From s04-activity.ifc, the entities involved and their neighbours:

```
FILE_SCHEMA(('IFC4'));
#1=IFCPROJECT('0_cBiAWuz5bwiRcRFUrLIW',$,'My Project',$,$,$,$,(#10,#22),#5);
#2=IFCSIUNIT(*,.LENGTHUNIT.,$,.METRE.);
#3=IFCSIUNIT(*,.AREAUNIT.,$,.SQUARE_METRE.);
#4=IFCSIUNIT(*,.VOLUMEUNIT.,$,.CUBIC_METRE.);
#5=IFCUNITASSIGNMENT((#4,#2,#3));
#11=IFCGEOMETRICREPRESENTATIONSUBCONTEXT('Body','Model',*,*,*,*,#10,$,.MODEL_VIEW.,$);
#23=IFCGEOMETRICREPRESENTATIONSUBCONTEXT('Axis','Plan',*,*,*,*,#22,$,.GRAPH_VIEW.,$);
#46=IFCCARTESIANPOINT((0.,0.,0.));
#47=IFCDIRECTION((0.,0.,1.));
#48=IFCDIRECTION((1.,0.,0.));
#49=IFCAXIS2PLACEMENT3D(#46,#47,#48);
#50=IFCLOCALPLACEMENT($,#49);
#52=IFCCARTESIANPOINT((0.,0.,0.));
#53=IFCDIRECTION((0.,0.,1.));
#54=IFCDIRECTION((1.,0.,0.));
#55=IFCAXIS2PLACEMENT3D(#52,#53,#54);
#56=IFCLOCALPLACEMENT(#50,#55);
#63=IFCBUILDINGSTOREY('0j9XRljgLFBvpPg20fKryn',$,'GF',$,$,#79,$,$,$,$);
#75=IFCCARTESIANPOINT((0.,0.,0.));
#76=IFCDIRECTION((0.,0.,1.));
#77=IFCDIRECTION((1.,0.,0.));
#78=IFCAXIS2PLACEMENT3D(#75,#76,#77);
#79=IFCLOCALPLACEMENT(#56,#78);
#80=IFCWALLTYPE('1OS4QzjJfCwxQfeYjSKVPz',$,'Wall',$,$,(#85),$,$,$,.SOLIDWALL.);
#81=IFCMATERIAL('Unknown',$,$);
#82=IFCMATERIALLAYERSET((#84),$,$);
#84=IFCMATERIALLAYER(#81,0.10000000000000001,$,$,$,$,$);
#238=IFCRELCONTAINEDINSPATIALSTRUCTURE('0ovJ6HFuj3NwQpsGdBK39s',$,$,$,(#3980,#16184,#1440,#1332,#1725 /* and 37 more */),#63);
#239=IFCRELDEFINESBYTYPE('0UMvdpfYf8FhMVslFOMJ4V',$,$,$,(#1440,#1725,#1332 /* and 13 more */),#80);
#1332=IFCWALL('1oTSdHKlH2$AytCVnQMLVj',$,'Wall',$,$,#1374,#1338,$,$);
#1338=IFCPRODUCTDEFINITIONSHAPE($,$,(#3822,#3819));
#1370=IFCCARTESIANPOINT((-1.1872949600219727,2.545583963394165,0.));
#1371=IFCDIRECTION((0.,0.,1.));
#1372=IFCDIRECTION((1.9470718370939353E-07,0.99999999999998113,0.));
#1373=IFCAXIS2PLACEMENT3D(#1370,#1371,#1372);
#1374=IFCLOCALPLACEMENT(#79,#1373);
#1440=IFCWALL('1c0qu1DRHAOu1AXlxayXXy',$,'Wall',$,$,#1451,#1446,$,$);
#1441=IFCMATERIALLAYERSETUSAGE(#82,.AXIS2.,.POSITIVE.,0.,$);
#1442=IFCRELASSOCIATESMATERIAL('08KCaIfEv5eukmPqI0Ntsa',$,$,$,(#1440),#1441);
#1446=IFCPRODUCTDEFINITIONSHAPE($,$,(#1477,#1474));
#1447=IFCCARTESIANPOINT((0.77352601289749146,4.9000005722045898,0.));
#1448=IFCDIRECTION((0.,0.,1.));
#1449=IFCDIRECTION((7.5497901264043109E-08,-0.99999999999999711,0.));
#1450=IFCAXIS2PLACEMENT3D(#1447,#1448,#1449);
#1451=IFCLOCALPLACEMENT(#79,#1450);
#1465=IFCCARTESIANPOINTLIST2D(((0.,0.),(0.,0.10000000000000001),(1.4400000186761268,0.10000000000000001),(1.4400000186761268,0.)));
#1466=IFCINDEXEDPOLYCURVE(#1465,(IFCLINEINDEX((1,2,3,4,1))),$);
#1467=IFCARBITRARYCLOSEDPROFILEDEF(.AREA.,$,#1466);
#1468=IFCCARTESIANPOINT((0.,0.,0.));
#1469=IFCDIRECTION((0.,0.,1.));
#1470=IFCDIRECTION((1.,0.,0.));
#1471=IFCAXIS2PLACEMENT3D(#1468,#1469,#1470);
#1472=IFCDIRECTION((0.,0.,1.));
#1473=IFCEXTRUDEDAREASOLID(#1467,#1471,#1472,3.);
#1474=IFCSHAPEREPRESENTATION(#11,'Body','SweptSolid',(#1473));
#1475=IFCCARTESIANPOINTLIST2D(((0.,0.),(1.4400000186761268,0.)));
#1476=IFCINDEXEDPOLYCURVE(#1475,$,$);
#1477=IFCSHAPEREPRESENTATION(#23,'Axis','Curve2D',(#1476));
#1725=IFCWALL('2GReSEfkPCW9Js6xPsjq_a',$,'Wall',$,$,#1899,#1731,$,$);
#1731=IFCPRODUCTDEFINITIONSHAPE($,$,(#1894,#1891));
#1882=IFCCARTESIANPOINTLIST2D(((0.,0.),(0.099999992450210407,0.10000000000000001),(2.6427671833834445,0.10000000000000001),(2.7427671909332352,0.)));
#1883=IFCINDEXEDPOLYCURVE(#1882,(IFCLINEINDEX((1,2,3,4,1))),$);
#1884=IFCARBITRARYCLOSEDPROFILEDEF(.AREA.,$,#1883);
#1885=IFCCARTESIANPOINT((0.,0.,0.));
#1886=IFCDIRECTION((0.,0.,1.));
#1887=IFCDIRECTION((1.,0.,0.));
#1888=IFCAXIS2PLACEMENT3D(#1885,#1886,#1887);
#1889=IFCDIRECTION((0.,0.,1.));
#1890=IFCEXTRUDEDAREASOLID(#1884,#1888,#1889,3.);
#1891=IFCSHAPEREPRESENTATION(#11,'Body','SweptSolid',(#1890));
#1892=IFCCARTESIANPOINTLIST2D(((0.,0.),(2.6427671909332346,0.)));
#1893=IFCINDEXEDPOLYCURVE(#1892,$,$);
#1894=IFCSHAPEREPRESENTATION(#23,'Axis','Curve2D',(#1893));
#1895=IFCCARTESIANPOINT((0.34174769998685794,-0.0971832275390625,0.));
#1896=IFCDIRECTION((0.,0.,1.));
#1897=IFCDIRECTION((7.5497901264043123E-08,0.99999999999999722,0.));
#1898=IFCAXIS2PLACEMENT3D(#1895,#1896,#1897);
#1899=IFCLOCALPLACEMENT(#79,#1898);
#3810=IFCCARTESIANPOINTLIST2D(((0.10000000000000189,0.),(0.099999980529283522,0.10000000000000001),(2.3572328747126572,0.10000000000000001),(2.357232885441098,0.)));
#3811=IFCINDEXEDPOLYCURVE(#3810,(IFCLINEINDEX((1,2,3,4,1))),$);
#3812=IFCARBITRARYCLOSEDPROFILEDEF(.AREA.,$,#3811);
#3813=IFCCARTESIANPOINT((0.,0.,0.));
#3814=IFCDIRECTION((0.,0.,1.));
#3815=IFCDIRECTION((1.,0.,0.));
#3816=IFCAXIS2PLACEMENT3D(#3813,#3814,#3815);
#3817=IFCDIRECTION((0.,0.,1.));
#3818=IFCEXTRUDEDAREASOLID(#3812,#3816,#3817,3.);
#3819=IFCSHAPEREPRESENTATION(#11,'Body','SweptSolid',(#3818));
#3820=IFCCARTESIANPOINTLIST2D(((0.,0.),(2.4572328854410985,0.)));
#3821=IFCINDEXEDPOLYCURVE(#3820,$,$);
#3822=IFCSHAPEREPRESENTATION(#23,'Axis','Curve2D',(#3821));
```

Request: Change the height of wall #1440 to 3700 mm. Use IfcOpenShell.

```python
import ifcopenshell
import ifcopenshell.geom
import ifcopenshell.util.representation
import ifcopenshell.util.shape
import ifcopenshell.util.unit

model = ifcopenshell.open("s04-activity.ifc")
unit_scale = ifcopenshell.util.unit.calculate_unit_scale(model)
settings = ifcopenshell.geom.settings()


def volume(element):
    """Net volume in cubic metres, openings subtracted."""
    shape = ifcopenshell.geom.create_shape(settings, element)
    return ifcopenshell.util.shape.get_volume(shape.geometry)


wall = model.by_guid("1c0qu1DRHAOu1AXlxayXXy")
before = volume(wall)

body = ifcopenshell.util.representation.get_representation(wall, "Model", "Body")
solid = body.Items[0]
old_height = solid.Depth
solid.Depth = 3.7 / unit_scale
after = volume(wall)

print(f"height {old_height:g} -> {solid.Depth:g}, volume {before:.3f} -> {after:.3f} m3")

model.write("s04-activity_updated.ifc")
```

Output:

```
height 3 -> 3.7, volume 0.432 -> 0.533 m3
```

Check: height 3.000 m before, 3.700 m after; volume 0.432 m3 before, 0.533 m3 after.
